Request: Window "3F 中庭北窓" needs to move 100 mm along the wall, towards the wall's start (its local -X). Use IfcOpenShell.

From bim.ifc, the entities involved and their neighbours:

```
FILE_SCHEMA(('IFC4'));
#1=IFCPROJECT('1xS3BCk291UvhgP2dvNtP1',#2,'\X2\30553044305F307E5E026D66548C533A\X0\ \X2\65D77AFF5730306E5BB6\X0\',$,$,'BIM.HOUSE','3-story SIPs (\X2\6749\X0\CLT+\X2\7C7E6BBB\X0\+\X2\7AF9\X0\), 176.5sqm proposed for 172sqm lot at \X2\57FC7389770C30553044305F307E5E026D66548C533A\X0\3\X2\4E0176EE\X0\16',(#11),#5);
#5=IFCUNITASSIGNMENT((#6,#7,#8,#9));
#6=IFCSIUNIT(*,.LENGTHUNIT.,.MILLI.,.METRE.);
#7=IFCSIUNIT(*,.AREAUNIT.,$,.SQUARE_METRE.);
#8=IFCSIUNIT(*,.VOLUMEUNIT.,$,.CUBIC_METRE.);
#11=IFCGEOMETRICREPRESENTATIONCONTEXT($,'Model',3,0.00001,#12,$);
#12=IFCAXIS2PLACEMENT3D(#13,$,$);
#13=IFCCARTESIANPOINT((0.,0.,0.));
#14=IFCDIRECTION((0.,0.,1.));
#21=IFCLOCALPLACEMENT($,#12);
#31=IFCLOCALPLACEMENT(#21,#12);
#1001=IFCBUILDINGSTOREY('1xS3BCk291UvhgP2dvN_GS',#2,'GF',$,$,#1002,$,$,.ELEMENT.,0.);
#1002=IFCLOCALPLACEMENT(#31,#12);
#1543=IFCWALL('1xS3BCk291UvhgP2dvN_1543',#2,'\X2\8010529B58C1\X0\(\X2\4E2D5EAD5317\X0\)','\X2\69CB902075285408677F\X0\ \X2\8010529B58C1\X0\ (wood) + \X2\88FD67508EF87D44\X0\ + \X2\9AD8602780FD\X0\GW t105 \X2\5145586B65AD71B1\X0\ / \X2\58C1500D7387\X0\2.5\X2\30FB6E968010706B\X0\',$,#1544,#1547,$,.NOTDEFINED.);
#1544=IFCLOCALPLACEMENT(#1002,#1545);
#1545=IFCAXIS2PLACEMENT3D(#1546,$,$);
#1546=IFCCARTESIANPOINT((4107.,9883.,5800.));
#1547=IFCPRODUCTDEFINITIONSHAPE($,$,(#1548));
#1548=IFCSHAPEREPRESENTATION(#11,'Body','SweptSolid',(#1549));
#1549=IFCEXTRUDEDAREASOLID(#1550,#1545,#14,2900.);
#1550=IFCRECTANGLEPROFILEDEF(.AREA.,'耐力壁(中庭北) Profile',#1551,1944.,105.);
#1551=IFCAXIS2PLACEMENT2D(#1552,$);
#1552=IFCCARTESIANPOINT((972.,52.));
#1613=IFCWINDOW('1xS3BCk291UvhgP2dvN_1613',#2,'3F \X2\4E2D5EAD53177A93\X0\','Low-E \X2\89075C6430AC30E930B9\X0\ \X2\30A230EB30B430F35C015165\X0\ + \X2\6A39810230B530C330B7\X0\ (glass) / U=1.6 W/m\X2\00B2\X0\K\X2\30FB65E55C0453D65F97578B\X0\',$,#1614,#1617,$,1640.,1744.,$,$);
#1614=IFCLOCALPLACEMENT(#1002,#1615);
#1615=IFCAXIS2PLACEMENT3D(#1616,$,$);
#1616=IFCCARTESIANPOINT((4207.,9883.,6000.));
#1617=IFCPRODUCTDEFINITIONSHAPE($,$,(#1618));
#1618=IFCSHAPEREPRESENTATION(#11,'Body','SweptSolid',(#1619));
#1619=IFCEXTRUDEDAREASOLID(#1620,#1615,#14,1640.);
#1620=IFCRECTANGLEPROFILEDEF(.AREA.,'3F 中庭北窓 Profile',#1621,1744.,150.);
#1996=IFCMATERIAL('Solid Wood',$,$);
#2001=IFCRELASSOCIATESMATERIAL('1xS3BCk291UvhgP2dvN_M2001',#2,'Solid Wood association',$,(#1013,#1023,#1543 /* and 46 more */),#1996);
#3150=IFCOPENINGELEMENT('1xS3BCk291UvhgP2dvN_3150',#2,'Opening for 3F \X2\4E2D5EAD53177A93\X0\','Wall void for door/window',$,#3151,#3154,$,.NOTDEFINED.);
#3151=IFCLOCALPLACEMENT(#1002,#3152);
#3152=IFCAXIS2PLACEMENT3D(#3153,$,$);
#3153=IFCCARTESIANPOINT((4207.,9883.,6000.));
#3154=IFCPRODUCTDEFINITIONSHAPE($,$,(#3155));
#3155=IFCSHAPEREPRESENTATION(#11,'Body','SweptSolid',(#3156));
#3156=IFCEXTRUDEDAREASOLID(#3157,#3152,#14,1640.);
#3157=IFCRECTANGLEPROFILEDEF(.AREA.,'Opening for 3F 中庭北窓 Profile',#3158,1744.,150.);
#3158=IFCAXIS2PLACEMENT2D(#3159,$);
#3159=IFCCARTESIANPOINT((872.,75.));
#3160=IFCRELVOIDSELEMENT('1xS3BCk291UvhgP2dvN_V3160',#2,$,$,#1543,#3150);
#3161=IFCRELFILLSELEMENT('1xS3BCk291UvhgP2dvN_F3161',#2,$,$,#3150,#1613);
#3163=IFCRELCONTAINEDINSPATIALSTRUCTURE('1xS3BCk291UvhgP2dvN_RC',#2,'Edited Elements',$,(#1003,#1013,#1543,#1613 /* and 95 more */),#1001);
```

```python
import ifcopenshell
import ifcopenshell.api.geometry
import ifcopenshell.util.placement

model = ifcopenshell.open("bim.ifc")

window = model.by_guid("1xS3BCk291UvhgP2dvN_1613")
opening = window.FillsVoids[0].RelatingOpeningElement
wall = opening.VoidsElements[0].RelatingBuildingElement

wall_matrix = ifcopenshell.util.placement.get_local_placement(wall.ObjectPlacement)
shift = wall_matrix[:3, 0] * -100.0
before = ifcopenshell.util.placement.get_local_placement(window.ObjectPlacement)[:3, 3].copy()

# The window is not placed relative to its opening, so move both.
for product in (opening, window):
    matrix = ifcopenshell.util.placement.get_local_placement(product.ObjectPlacement)
    matrix[:3, 3] += shift
    ifcopenshell.api.geometry.edit_object_placement(model, product=product, matrix=matrix, is_si=False)

after = ifcopenshell.util.placement.get_local_placement(window.ObjectPlacement)[:3, 3]
print("window moved by", (after - before).round(3) + 0.0)

model.write("bim_edited.ifc")
```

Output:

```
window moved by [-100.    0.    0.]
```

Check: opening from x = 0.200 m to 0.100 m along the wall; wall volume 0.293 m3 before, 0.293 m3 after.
